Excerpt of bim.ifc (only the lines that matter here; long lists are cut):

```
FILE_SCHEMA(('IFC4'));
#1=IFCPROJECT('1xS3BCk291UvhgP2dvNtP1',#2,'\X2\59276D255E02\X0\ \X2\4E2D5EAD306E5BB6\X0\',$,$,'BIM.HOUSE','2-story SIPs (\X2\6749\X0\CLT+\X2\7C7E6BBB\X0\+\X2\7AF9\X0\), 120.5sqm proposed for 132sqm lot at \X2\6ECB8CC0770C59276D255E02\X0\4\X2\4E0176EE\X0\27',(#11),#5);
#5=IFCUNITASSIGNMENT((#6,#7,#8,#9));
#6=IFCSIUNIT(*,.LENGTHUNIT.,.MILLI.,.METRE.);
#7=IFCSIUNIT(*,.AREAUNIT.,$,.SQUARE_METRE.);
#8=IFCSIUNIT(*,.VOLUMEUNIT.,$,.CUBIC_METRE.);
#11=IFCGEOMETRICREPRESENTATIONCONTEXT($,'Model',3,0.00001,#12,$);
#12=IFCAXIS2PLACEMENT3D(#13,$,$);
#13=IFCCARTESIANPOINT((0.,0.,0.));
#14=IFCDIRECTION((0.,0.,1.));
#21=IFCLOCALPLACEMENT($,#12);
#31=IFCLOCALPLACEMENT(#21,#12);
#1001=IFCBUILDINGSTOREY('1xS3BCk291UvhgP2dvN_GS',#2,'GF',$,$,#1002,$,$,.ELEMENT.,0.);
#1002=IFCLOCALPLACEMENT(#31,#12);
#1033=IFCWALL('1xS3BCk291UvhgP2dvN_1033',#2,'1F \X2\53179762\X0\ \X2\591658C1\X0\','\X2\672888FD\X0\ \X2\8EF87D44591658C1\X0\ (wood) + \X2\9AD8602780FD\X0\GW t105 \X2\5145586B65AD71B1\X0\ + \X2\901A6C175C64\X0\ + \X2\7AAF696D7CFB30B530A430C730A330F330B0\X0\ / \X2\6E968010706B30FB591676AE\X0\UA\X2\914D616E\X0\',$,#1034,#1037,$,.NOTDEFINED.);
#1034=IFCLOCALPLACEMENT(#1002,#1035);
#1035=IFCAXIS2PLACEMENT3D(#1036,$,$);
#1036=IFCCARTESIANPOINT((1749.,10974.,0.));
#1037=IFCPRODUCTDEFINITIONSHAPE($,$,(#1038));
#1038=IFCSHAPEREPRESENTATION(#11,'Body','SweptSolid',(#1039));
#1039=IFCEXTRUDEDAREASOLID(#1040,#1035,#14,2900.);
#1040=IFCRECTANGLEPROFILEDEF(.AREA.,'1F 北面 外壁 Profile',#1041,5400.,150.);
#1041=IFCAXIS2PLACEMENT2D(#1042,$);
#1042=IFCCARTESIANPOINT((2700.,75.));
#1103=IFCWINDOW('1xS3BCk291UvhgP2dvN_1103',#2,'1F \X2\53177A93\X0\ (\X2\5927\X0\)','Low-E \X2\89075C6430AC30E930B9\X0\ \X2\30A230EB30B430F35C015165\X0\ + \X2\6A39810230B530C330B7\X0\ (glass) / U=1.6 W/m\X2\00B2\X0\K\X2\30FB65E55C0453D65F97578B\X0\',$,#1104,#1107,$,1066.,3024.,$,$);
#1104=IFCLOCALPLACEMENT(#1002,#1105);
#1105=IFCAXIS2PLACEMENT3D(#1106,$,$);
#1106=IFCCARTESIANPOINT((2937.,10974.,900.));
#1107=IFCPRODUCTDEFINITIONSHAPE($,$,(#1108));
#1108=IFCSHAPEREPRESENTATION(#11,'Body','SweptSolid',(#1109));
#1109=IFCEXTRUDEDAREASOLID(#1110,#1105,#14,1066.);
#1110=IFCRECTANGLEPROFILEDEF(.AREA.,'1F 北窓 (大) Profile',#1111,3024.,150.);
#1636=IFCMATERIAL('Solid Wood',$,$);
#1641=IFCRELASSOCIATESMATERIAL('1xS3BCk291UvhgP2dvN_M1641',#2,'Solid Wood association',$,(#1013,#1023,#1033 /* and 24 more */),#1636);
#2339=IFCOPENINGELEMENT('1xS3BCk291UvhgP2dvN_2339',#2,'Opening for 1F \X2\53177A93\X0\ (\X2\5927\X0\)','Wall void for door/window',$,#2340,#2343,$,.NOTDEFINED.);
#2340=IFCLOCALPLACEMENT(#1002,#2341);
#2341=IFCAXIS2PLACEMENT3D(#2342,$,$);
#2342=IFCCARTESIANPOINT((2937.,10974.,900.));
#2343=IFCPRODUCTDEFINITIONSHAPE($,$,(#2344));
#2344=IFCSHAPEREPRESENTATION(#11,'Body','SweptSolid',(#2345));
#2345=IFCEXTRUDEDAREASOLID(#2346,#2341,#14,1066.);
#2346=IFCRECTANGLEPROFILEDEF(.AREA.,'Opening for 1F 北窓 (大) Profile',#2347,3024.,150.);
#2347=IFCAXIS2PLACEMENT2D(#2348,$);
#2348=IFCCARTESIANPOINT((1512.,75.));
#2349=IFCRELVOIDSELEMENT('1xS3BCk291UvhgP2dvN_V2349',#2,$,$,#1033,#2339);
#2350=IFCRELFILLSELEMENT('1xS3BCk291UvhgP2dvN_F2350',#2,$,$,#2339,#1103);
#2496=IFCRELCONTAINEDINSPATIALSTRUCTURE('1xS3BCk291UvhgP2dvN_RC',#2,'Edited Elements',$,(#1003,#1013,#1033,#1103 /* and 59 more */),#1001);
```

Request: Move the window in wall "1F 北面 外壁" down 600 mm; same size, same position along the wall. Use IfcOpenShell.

```python
import numpy as np
import ifcopenshell
import ifcopenshell.api.geometry
import ifcopenshell.util.placement
import ifcopenshell.util.unit

model = ifcopenshell.open("bim.ifc")
unit_scale = ifcopenshell.util.unit.calculate_unit_scale(model)

window = model.by_guid("1xS3BCk291UvhgP2dvN_1103")
opening = window.FillsVoids[0].RelatingOpeningElement
dz = -0.6 / unit_scale

shift = np.array([0.0, 0.0, dz])
# The window is not placed relative to its opening, so move both.
for product in (opening, window):
    matrix = ifcopenshell.util.placement.get_local_placement(product.ObjectPlacement)
    matrix[:3, 3] += shift
    ifcopenshell.api.geometry.edit_object_placement(model, product=product, matrix=matrix, is_si=False)

print(f"moved by {dz * unit_scale:+.3f} m")

model.write("bim_rev.ifc")
```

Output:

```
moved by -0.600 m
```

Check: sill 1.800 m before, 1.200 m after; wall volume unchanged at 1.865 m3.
